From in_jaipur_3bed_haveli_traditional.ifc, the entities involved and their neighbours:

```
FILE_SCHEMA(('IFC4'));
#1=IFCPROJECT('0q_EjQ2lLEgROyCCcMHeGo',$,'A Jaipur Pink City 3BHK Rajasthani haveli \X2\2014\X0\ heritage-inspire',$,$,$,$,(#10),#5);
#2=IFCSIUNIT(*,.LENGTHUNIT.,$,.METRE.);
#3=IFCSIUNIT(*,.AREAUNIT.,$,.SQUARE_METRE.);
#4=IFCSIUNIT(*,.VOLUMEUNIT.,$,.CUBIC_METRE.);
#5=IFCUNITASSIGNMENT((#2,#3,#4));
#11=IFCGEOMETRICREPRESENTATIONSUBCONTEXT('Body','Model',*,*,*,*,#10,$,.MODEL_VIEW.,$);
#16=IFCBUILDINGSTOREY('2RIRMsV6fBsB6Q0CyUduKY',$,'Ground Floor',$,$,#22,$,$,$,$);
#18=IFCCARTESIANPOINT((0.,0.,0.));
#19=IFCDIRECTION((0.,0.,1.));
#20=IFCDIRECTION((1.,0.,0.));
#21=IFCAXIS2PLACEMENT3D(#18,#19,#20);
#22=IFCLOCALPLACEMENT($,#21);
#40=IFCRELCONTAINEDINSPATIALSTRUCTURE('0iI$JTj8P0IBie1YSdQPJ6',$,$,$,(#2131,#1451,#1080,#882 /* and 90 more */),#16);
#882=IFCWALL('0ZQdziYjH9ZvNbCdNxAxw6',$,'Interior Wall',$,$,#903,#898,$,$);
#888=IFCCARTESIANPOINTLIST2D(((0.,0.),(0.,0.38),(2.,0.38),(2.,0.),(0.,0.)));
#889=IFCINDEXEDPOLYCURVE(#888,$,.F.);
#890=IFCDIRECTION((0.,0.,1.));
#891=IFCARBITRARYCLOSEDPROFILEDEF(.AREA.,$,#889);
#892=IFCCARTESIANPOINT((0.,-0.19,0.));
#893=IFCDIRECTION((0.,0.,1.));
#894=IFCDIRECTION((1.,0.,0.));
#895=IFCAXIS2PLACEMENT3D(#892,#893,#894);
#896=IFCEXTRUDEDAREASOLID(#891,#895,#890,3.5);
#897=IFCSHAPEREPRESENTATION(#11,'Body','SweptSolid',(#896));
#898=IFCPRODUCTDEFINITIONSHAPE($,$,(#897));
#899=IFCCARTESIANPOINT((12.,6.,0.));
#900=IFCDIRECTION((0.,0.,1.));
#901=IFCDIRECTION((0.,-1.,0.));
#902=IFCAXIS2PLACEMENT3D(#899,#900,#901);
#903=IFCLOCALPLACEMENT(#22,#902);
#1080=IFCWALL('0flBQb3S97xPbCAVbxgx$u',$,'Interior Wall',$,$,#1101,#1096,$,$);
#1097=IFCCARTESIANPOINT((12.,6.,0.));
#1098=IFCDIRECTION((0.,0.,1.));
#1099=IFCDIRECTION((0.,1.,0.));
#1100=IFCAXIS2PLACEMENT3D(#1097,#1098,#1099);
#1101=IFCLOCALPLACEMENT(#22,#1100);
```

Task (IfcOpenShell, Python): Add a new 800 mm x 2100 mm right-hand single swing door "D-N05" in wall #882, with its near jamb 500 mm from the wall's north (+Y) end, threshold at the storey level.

```python
import numpy as np
import ifcopenshell
import ifcopenshell.api.feature
import ifcopenshell.api.geometry
import ifcopenshell.api.root
import ifcopenshell.api.spatial
import ifcopenshell.geom
import ifcopenshell.util.element
import ifcopenshell.util.placement
import ifcopenshell.util.representation
import ifcopenshell.util.shape
import ifcopenshell.util.unit

model = ifcopenshell.open("in_jaipur_3bed_haveli_traditional.ifc")
unit_scale = ifcopenshell.util.unit.calculate_unit_scale(model)
settings = ifcopenshell.geom.settings()


def volume(element):
    """Net volume in cubic metres, openings subtracted."""
    shape = ifcopenshell.geom.create_shape(settings, element)
    return ifcopenshell.util.shape.get_volume(shape.geometry)


wall = model.by_guid("0ZQdziYjH9ZvNbCdNxAxw6")
storey = ifcopenshell.util.element.get_container(wall, ifc_class="IfcBuildingStorey")
context = ifcopenshell.util.representation.get_context(model, "Model", "Body", "MODEL_VIEW")
before = volume(wall)

width, height, from_end, sill = 0.8, 2.1, 0.5, 0.0  # metres

# The wall runs along its own X axis, and the end named is its -X end.
wall_shape = ifcopenshell.geom.create_shape(settings, wall)
x, y, z = ifcopenshell.util.shape.get_vertices(wall_shape.geometry).T
start = x.min() + from_end
face, thickness = float(y.min()), float(y.max() - y.min())
wall_matrix = ifcopenshell.util.placement.get_local_placement(wall.ObjectPlacement)
level = ifcopenshell.util.placement.get_local_placement(storey.ObjectPlacement)[2, 3]


def in_wall(x, y):
    """Placement at x, y metres in the wall's axes, at sill height."""
    matrix = wall_matrix.copy()
    matrix[:, 3] = wall_matrix @ np.array([x / unit_scale, y / unit_scale, 0.0, 1.0])
    matrix[2, 3] = level + sill / unit_scale
    return matrix


# Opening: a box that overshoots both wall faces by 50 mm.
opening = ifcopenshell.api.root.create_entity(model, ifc_class="IfcOpeningElement", predefined_type="OPENING")
box = ifcopenshell.api.geometry.add_wall_representation(
    model, context=context, length=width, height=height, thickness=thickness + 0.1
)
ifcopenshell.api.geometry.assign_representation(model, product=opening, representation=box)
ifcopenshell.api.geometry.edit_object_placement(model, product=opening, matrix=in_wall(start, face - 0.05), is_si=False)
ifcopenshell.api.feature.add_feature(model, feature=opening, element=wall)

door = ifcopenshell.api.root.create_entity(model, ifc_class="IfcDoor", name="D-N05", predefined_type="DOOR")
door.OverallWidth, door.OverallHeight = width / unit_scale, height / unit_scale
door.OperationType = "SINGLE_SWING_RIGHT"
body = ifcopenshell.api.geometry.add_door_representation(
    model,
    context=context,
    overall_width=door.OverallWidth,
    overall_height=door.OverallHeight,
    operation_type="SINGLE_SWING_RIGHT",
    lining_properties={"LiningDepth": thickness / unit_scale, "ThresholdDepth": thickness / unit_scale},
)
ifcopenshell.api.geometry.assign_representation(model, product=door, representation=body)
ifcopenshell.api.spatial.assign_container(model, products=[door], relating_structure=storey)
ifcopenshell.api.feature.add_filling(model, opening=opening, element=door)

# The lining spans the wall, so the door starts at the wall face.
ifcopenshell.api.geometry.edit_object_placement(model, product=door, matrix=in_wall(start, face), is_si=False)

after = volume(wall)

print(f"wall volume {before:.3f} -> {after:.3f} m3")

model.write("in_jaipur_3bed_haveli_traditional_v2.ifc")
```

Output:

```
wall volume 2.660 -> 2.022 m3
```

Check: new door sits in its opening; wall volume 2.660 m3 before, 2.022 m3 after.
